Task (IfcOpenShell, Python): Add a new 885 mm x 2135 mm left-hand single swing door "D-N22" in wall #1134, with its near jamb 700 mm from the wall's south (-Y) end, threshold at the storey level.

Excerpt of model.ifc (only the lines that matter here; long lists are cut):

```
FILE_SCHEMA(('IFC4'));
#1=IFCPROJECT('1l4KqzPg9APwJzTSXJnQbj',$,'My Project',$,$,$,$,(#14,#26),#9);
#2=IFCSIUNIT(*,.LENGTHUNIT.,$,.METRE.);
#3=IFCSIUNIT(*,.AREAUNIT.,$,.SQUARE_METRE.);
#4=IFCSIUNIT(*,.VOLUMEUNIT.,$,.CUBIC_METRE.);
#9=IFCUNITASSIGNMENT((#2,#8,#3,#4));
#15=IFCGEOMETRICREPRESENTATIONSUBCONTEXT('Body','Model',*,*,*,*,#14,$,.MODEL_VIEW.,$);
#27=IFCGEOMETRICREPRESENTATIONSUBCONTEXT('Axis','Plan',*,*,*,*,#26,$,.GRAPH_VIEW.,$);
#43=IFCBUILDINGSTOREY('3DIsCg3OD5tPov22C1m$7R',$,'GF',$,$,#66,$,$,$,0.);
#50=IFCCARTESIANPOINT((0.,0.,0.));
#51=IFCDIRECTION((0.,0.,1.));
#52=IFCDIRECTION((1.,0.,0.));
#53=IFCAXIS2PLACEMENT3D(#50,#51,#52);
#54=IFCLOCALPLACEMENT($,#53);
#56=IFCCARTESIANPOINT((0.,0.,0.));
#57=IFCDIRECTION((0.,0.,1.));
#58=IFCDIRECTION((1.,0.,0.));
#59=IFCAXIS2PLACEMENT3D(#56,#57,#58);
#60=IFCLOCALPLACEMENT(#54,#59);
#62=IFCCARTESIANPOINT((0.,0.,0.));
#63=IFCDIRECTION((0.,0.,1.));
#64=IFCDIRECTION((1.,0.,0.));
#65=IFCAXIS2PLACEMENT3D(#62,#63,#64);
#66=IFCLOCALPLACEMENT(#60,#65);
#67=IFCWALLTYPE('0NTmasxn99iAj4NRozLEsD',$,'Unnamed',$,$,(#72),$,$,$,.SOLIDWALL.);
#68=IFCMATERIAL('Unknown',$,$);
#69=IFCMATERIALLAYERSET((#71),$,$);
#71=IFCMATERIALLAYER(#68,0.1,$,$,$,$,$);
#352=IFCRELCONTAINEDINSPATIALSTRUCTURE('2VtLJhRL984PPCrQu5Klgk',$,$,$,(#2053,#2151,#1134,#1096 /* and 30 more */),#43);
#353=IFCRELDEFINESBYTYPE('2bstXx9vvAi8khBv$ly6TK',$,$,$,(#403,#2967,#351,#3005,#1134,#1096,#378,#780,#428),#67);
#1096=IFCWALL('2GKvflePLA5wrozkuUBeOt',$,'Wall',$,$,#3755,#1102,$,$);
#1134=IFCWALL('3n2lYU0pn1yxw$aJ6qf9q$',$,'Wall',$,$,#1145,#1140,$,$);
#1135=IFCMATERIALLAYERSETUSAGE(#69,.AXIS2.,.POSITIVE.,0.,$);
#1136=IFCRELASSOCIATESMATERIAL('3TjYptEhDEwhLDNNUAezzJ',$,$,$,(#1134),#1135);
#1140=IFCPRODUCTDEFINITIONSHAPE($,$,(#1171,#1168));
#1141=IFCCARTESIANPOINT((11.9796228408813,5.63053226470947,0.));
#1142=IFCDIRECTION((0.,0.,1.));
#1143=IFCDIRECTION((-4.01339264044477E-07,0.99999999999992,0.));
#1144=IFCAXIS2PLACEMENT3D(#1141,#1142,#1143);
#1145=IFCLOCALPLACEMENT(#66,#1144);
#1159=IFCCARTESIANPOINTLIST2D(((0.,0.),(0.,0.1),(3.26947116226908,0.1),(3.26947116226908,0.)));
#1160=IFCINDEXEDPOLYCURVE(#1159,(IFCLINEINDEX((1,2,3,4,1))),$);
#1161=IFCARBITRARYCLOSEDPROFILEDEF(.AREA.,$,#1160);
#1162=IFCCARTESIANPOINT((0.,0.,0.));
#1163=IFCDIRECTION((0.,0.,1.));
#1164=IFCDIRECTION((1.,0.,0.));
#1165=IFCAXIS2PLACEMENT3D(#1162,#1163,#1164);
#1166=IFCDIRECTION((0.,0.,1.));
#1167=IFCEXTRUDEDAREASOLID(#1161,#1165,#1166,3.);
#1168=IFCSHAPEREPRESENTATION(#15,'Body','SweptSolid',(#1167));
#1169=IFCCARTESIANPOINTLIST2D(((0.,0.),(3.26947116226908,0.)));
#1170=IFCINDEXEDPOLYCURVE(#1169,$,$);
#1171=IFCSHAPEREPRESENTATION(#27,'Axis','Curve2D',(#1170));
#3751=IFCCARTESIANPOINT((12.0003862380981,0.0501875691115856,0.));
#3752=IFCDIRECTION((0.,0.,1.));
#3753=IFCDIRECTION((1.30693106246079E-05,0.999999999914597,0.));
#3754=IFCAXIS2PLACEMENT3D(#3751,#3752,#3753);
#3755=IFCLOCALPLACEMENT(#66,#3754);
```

```python
import numpy as np
import ifcopenshell
import ifcopenshell.api.feature
import ifcopenshell.api.geometry
import ifcopenshell.api.root
import ifcopenshell.api.spatial
import ifcopenshell.geom
import ifcopenshell.util.element
import ifcopenshell.util.placement
import ifcopenshell.util.representation
import ifcopenshell.util.shape
import ifcopenshell.util.unit

model = ifcopenshell.open("model.ifc")
unit_scale = ifcopenshell.util.unit.calculate_unit_scale(model)
settings = ifcopenshell.geom.settings()


def volume(element):
    """Net volume in cubic metres, openings subtracted."""
    shape = ifcopenshell.geom.create_shape(settings, element)
    return ifcopenshell.util.shape.get_volume(shape.geometry)


wall = model.by_guid("3n2lYU0pn1yxw$aJ6qf9q$")
storey = ifcopenshell.util.element.get_container(wall, ifc_class="IfcBuildingStorey")
context = ifcopenshell.util.representation.get_context(model, "Model", "Body", "MODEL_VIEW")
before = volume(wall)

width, height, from_end, sill = 0.885, 2.135, 0.7, 0.0  # metres

# The wall runs along its own X axis, and the end named is its -X end.
wall_shape = ifcopenshell.geom.create_shape(settings, wall)
x, y, z = ifcopenshell.util.shape.get_vertices(wall_shape.geometry).T
start = x.min() + from_end
face, thickness = float(y.min()), float(y.max() - y.min())
wall_matrix = ifcopenshell.util.placement.get_local_placement(wall.ObjectPlacement)
level = ifcopenshell.util.placement.get_local_placement(storey.ObjectPlacement)[2, 3]


def in_wall(x, y):
    """Placement at x, y metres in the wall's axes, at sill height."""
    matrix = wall_matrix.copy()
    matrix[:, 3] = wall_matrix @ np.array([x / unit_scale, y / unit_scale, 0.0, 1.0])
    matrix[2, 3] = level + sill / unit_scale
    return matrix


# Opening: a box that overshoots both wall faces by 50 mm.
opening = ifcopenshell.api.root.create_entity(model, ifc_class="IfcOpeningElement", predefined_type="OPENING")
box = ifcopenshell.api.geometry.add_wall_representation(
    model, context=context, length=width, height=height, thickness=thickness + 0.1
)
ifcopenshell.api.geometry.assign_representation(model, product=opening, representation=box)
ifcopenshell.api.geometry.edit_object_placement(model, product=opening, matrix=in_wall(start, face - 0.05), is_si=False)
ifcopenshell.api.feature.add_feature(model, feature=opening, element=wall)

door = ifcopenshell.api.root.create_entity(model, ifc_class="IfcDoor", name="D-N22", predefined_type="DOOR")
door.OverallWidth, door.OverallHeight = width / unit_scale, height / unit_scale
door.OperationType = "SINGLE_SWING_LEFT"
body = ifcopenshell.api.geometry.add_door_representation(
    model,
    context=context,
    overall_width=door.OverallWidth,
    overall_height=door.OverallHeight,
    operation_type="SINGLE_SWING_LEFT",
    lining_properties={"LiningDepth": thickness / unit_scale, "ThresholdDepth": thickness / unit_scale},
)
ifcopenshell.api.geometry.assign_representation(model, product=door, representation=body)
ifcopenshell.api.spatial.assign_container(model, products=[door], relating_structure=storey)
ifcopenshell.api.feature.add_filling(model, opening=opening, element=door)

# The lining spans the wall, so the door starts at the wall face.
ifcopenshell.api.geometry.edit_object_placement(model, product=door, matrix=in_wall(start, face), is_si=False)

after = volume(wall)

print(f"wall volume {before:.3f} -> {after:.3f} m3")

model.write("model-out.ifc")
```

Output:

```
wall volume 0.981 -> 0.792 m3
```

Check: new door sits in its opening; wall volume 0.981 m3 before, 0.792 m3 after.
